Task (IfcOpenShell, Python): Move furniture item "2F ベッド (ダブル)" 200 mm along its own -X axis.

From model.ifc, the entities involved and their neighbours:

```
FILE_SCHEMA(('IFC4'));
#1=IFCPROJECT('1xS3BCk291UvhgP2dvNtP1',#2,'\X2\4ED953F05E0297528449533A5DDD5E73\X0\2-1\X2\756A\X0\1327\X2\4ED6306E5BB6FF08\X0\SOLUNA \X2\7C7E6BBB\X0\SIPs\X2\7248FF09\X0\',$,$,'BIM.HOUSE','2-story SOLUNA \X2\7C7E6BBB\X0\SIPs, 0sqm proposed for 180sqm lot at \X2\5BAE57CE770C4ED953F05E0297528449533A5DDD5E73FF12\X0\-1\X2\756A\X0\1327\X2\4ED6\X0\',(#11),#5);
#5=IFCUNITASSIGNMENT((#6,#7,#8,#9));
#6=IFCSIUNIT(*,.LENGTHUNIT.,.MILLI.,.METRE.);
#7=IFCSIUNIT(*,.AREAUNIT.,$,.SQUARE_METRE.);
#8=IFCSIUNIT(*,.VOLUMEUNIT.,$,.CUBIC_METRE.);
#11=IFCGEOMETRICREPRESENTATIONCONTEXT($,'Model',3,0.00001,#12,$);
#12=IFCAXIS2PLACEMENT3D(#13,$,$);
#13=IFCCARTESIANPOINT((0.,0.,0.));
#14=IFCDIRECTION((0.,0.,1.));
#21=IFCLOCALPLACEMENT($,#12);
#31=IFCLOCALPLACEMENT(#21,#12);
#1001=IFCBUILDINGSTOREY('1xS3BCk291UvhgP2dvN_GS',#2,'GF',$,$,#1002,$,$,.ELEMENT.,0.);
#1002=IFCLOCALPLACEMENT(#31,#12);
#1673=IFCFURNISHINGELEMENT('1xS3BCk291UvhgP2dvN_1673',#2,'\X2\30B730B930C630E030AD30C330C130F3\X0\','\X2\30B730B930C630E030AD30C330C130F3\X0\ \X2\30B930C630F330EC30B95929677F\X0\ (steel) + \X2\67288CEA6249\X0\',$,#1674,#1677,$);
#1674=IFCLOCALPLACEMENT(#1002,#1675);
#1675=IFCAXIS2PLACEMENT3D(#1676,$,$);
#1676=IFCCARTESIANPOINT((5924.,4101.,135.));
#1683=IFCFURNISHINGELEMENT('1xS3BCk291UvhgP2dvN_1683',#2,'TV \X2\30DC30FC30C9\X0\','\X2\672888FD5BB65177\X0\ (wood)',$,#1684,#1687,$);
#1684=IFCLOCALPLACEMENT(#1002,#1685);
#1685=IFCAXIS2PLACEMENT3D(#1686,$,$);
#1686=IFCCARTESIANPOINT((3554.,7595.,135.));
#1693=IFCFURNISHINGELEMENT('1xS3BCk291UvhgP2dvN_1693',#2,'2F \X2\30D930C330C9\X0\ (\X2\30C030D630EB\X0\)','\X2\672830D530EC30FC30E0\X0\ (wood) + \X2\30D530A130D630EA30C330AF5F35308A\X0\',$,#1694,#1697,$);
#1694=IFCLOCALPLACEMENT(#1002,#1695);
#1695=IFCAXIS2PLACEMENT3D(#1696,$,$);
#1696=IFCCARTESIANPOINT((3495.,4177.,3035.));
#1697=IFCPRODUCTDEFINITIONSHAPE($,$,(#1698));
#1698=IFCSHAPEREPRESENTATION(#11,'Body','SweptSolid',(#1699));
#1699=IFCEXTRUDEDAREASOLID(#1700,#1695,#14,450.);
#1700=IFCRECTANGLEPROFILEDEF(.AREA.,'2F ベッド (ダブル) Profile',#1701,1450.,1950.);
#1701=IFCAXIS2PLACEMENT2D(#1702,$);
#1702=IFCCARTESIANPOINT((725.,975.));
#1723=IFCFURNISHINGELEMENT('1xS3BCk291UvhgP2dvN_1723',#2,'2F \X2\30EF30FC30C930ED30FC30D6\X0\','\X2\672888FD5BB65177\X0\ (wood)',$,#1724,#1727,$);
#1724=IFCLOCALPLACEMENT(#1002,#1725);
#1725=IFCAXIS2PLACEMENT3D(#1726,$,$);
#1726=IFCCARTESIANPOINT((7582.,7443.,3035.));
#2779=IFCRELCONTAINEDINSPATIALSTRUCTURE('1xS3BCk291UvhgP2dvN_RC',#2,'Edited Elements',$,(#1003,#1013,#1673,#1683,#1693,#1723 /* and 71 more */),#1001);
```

```python
import ifcopenshell
import ifcopenshell.api.geometry
import ifcopenshell.util.placement
import ifcopenshell.util.unit

model = ifcopenshell.open("model.ifc")
unit_scale = ifcopenshell.util.unit.calculate_unit_scale(model)

item = model.by_guid("1xS3BCk291UvhgP2dvN_1693")
matrix = ifcopenshell.util.placement.get_local_placement(item.ObjectPlacement)
matrix[:3, 3] -= matrix[:3, 0] * 0.2 / unit_scale
ifcopenshell.api.geometry.edit_object_placement(model, product=item, matrix=matrix, is_si=False)

print(ifcopenshell.util.placement.get_local_placement(item.ObjectPlacement).round(3) + 0.0)

model.write("model-out.ifc")
```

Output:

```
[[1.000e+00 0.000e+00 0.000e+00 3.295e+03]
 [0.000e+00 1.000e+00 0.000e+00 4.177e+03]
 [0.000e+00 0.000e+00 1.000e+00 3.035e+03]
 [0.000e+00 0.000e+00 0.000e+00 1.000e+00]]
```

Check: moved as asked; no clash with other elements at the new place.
